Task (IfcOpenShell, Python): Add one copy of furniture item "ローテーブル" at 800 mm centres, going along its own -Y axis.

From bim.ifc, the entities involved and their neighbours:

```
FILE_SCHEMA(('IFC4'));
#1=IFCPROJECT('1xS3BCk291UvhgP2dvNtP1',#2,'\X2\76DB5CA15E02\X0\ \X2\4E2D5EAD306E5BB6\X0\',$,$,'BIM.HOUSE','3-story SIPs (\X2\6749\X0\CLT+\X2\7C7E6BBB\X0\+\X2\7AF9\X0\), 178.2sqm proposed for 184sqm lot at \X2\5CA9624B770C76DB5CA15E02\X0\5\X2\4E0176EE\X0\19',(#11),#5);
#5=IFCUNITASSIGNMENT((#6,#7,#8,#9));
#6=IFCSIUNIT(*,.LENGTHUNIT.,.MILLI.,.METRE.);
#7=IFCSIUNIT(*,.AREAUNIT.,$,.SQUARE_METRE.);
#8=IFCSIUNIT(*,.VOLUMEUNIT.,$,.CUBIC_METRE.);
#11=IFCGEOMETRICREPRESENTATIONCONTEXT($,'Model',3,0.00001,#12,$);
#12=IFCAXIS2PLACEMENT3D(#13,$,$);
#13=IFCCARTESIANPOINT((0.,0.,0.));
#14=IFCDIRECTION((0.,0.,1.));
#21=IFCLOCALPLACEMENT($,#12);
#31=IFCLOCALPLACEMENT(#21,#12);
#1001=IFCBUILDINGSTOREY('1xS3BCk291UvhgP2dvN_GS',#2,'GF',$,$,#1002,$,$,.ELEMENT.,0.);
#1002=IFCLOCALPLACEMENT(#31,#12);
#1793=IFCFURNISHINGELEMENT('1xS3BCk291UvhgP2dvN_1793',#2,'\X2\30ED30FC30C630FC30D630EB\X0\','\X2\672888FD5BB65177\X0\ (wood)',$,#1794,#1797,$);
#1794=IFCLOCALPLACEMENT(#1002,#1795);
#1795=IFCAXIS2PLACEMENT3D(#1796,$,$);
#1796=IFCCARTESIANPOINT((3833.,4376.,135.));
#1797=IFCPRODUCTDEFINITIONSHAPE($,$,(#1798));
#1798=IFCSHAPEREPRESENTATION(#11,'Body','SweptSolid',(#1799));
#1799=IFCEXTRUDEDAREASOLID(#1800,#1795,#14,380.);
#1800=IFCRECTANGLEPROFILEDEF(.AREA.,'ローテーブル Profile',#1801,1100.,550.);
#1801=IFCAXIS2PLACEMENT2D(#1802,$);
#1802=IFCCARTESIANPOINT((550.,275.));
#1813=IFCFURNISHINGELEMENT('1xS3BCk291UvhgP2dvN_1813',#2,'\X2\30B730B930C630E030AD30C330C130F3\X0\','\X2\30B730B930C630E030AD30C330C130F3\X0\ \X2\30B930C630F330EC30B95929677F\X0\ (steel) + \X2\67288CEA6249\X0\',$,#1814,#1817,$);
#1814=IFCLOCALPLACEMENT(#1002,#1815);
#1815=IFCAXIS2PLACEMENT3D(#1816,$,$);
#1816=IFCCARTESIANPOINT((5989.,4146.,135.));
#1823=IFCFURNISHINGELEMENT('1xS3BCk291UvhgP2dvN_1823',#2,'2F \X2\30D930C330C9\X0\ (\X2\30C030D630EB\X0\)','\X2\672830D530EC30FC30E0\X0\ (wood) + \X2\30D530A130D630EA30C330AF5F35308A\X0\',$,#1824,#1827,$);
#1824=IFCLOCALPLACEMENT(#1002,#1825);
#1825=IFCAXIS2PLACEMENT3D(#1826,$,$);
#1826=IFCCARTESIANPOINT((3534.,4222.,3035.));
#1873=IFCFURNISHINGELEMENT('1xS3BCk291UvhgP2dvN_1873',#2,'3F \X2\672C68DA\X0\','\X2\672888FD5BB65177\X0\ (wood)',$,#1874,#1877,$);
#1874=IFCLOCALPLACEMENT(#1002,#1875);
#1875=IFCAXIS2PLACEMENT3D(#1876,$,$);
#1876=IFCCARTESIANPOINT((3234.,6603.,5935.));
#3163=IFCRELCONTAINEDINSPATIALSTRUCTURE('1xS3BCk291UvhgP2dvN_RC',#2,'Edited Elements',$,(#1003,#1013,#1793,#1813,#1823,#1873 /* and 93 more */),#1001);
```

```python
import ifcopenshell
import ifcopenshell.api.geometry
import ifcopenshell.api.root
import ifcopenshell.util.element
import ifcopenshell.util.placement
import ifcopenshell.util.unit

model = ifcopenshell.open("bim.ifc")
unit_scale = ifcopenshell.util.unit.calculate_unit_scale(model)


def reuse_history(source, copy):
    """copy_class also copies each property set's owner history, people and application; keep the originals."""
    for rel in copy.IsDefinedBy:
        if rel.is_a("IfcRelDefinesByProperties") and (history := rel.RelatingPropertyDefinition.OwnerHistory):
            rel.RelatingPropertyDefinition.OwnerHistory = source.OwnerHistory
            ifcopenshell.util.element.remove_deep2(model, history)


source = model.by_guid("1xS3BCk291UvhgP2dvN_1793")
base = ifcopenshell.util.placement.get_local_placement(source.ObjectPlacement)
step = -base[:3, 1] * 0.8 / unit_scale

for i in range(1, 2):
    copy = ifcopenshell.api.root.copy_class(model, product=source)
    copy.Representation = ifcopenshell.util.element.copy_deep(
        model, source.Representation, exclude=["IfcGeometricRepresentationContext", "IfcRepresentationMap"]
    )
    reuse_history(source, copy)
    matrix = base.copy()
    matrix[:3, 3] += i * step
    print("added at", matrix[:3, 3].round(3) + 0.0)
    ifcopenshell.api.geometry.edit_object_placement(model, product=copy, matrix=matrix, is_si=False)

model.write("bim-out.ifc")
```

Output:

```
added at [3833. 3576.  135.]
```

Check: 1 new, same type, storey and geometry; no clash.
